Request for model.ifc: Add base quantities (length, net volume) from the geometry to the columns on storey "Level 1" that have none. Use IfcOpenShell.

First a look at what the model holds.

```python
import ifcopenshell
import ifcopenshell.util.element
import ifcopenshell.util.unit

model = ifcopenshell.open("model.ifc")
print(model.schema)
for unit_type in ("LENGTHUNIT", "AREAUNIT", "VOLUMEUNIT"):
    print(unit_type, ifcopenshell.util.unit.calculate_unit_scale(model, unit_type))
storey = next(s for s in model.by_type("IfcBuildingStorey") if s.Name == "Level 1")
columns = [e for e in ifcopenshell.util.element.get_decomposition(storey) if e.is_a("IfcColumn")]
for e in sorted(columns, key=lambda e: e.id()):
    print(e.id(), e.is_a(), e.Name, list(ifcopenshell.util.element.get_psets(e, qtos_only=True)), sep=" | ")
```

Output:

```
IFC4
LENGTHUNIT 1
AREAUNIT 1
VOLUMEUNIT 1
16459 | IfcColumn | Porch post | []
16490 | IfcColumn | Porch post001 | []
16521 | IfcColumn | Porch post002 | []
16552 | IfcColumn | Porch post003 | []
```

```python
import ifcopenshell
import ifcopenshell.api.pset
import ifcopenshell.geom
import ifcopenshell.util.element
import ifcopenshell.util.shape
import ifcopenshell.util.unit

model = ifcopenshell.open("model.ifc")
unit_scale = ifcopenshell.util.unit.calculate_unit_scale(model)
volume_scale = ifcopenshell.util.unit.calculate_unit_scale(model, "VOLUMEUNIT")
settings = ifcopenshell.geom.settings()

storey = next(s for s in model.by_type("IfcBuildingStorey") if s.Name == "Level 1")
columns = [e for e in ifcopenshell.util.element.get_decomposition(storey) if e.is_a("IfcColumn")]

for e in sorted(columns, key=lambda e: e.id()):
    if ifcopenshell.util.element.get_psets(e, qtos_only=True, should_inherit=False):
        continue
    # Geometry comes back in metres, in the element's own axes.
    shape = ifcopenshell.geom.create_shape(settings, e)
    values = {
        "Length": ifcopenshell.util.shape.get_z(shape.geometry) / unit_scale,
        "NetVolume": ifcopenshell.util.shape.get_volume(shape.geometry) / volume_scale,
    }
    qto = ifcopenshell.api.pset.add_qto(model, product=e, name="Qto_ColumnBaseQuantities")
    ifcopenshell.api.pset.edit_qto(model, qto=qto, properties=values)
    print(e.id(), {k: round(v, 3) for k, v in values.items()})

model.write("model_v2.ifc")
```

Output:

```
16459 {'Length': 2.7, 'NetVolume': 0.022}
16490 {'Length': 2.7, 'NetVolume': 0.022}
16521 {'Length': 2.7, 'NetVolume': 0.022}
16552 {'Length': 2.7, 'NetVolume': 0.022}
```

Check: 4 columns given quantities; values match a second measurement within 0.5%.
